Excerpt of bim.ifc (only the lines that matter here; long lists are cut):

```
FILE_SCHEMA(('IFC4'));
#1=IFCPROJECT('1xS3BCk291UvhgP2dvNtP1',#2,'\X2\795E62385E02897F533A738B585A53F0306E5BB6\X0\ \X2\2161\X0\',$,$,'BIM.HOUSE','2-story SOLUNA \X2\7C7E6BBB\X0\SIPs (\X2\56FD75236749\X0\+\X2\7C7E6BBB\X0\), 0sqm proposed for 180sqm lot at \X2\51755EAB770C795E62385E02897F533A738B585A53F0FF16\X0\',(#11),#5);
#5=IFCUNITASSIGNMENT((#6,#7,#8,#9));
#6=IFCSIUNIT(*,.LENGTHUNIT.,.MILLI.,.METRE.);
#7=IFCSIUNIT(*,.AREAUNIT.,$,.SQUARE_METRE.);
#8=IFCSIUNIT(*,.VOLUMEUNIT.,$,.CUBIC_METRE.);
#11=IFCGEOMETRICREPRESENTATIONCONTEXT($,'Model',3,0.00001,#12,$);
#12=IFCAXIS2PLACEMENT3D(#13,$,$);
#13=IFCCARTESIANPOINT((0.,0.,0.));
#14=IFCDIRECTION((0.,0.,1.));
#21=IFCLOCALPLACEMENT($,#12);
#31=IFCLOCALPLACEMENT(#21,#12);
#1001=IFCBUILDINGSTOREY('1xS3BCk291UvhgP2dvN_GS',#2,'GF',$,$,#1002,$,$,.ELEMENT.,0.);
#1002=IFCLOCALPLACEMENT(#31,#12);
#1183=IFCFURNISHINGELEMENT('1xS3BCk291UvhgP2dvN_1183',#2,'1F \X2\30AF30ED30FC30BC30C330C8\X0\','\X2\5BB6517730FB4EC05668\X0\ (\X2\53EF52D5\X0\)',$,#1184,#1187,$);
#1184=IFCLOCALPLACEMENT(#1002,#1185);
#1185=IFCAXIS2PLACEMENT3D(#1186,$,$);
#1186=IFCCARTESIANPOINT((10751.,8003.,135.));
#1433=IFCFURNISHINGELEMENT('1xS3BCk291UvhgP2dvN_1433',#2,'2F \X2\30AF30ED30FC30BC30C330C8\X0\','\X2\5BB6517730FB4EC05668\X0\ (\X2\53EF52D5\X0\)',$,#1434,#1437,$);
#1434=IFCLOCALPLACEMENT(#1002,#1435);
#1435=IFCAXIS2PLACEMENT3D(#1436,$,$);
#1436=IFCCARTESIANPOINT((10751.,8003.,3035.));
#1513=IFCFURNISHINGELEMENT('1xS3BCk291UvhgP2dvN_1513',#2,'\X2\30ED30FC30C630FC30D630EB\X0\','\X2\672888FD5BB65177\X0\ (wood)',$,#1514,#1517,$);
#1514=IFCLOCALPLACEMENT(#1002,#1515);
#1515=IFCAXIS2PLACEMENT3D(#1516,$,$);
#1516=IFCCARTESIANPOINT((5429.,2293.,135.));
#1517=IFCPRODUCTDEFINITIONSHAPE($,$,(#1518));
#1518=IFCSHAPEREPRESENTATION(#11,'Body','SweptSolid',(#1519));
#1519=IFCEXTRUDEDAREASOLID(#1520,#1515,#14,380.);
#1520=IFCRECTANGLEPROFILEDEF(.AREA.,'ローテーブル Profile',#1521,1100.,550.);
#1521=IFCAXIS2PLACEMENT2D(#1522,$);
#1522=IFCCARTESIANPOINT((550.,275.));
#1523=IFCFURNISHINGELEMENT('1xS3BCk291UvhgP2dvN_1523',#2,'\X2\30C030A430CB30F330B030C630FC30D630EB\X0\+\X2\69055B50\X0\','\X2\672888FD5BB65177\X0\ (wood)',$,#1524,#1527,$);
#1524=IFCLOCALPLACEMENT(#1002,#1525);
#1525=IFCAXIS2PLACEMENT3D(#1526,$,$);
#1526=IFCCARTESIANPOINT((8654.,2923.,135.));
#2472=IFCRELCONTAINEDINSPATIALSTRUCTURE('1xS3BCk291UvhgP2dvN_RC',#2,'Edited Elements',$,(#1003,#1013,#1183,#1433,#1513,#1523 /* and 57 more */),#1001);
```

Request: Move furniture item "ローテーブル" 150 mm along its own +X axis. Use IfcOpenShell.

```python
import ifcopenshell
import ifcopenshell.api.geometry
import ifcopenshell.util.placement

model = ifcopenshell.open("bim.ifc")

item = model.by_guid("1xS3BCk291UvhgP2dvN_1513")
matrix = ifcopenshell.util.placement.get_local_placement(item.ObjectPlacement)
matrix[:3, 3] += matrix[:3, 0] * 150.0
ifcopenshell.api.geometry.edit_object_placement(model, product=item, matrix=matrix, is_si=False)

print(ifcopenshell.util.placement.get_local_placement(item.ObjectPlacement).round(3) + 0.0)

model.write("bim_edited.ifc")
```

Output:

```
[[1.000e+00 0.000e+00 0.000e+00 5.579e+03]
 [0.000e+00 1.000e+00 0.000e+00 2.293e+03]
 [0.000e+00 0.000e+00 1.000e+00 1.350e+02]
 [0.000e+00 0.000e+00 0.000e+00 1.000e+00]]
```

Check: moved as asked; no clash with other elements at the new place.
